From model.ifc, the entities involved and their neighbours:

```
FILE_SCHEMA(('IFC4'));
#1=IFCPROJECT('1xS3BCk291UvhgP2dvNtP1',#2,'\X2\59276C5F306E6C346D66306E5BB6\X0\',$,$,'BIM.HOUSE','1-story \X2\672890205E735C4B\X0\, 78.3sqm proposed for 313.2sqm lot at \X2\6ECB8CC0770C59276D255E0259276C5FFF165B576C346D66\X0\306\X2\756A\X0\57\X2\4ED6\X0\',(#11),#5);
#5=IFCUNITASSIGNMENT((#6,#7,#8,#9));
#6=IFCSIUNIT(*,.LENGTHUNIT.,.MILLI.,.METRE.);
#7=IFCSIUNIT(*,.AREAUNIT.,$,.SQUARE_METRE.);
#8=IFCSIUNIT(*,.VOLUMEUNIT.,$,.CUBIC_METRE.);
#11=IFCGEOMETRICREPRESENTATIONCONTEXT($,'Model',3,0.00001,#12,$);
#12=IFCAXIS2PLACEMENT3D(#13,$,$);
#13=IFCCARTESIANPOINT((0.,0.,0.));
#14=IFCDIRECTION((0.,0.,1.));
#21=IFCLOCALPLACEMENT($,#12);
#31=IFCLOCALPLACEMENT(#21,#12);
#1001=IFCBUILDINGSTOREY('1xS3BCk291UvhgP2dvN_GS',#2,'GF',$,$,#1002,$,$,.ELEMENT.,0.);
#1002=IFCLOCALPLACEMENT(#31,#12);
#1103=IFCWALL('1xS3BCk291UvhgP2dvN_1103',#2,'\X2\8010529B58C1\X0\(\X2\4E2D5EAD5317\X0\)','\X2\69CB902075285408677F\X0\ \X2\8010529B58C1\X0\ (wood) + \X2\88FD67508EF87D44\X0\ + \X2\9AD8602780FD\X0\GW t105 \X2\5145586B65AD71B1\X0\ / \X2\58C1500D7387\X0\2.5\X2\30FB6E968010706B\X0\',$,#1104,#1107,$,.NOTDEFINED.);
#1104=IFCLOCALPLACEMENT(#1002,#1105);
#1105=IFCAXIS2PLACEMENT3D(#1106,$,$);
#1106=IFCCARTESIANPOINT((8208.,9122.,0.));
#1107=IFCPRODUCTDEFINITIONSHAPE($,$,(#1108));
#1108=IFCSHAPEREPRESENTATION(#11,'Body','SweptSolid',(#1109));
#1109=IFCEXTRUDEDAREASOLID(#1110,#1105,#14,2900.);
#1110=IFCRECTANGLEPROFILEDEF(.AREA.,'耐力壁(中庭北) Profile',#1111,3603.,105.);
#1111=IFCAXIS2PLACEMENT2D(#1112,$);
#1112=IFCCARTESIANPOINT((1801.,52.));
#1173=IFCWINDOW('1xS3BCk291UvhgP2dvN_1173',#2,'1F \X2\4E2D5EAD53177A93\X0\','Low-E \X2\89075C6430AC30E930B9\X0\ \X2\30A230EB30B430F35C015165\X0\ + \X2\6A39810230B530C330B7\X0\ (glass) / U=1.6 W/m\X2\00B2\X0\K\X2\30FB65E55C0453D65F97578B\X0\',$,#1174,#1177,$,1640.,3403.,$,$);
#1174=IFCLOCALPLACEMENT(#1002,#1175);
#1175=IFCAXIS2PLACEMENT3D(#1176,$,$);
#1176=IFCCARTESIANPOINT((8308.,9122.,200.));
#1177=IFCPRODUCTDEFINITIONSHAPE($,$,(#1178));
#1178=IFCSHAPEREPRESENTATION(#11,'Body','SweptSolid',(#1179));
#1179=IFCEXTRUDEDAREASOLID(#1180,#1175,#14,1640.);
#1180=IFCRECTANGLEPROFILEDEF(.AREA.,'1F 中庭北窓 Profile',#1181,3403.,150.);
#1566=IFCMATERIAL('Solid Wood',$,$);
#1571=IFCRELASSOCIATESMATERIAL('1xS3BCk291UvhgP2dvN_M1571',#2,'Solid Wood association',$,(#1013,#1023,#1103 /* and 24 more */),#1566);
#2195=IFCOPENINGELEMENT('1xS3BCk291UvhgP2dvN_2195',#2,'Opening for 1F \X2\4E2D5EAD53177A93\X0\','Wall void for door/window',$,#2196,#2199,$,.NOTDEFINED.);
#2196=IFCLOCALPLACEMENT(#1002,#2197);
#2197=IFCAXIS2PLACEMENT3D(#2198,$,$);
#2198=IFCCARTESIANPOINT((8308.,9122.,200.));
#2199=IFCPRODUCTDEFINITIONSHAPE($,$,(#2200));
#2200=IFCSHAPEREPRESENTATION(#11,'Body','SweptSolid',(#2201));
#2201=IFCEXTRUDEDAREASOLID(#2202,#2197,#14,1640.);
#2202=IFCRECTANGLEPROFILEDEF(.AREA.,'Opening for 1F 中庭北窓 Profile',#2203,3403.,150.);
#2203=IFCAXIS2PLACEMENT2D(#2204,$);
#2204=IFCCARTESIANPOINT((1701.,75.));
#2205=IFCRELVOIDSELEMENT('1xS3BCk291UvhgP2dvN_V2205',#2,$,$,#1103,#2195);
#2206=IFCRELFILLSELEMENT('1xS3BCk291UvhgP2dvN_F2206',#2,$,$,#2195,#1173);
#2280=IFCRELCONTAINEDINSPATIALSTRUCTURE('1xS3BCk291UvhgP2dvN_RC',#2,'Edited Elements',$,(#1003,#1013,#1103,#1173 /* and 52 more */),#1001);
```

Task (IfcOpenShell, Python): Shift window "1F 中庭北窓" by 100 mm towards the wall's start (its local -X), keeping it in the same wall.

```python
import ifcopenshell
import ifcopenshell.api.geometry
import ifcopenshell.util.placement
import ifcopenshell.util.unit

model = ifcopenshell.open("model.ifc")
unit_scale = ifcopenshell.util.unit.calculate_unit_scale(model)

window = model.by_guid("1xS3BCk291UvhgP2dvN_1173")
opening = window.FillsVoids[0].RelatingOpeningElement
wall = opening.VoidsElements[0].RelatingBuildingElement

wall_matrix = ifcopenshell.util.placement.get_local_placement(wall.ObjectPlacement)
shift = wall_matrix[:3, 0] * -0.1 / unit_scale
before = ifcopenshell.util.placement.get_local_placement(window.ObjectPlacement)[:3, 3].copy()

# The window is not placed relative to its opening, so move both.
for product in (opening, window):
    matrix = ifcopenshell.util.placement.get_local_placement(product.ObjectPlacement)
    matrix[:3, 3] += shift
    ifcopenshell.api.geometry.edit_object_placement(model, product=product, matrix=matrix, is_si=False)

after = ifcopenshell.util.placement.get_local_placement(window.ObjectPlacement)[:3, 3]
print("window moved by", (after - before).round(3) + 0.0)

model.write("model_edited.ifc")
```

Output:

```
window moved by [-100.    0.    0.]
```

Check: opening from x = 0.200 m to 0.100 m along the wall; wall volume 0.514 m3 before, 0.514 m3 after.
